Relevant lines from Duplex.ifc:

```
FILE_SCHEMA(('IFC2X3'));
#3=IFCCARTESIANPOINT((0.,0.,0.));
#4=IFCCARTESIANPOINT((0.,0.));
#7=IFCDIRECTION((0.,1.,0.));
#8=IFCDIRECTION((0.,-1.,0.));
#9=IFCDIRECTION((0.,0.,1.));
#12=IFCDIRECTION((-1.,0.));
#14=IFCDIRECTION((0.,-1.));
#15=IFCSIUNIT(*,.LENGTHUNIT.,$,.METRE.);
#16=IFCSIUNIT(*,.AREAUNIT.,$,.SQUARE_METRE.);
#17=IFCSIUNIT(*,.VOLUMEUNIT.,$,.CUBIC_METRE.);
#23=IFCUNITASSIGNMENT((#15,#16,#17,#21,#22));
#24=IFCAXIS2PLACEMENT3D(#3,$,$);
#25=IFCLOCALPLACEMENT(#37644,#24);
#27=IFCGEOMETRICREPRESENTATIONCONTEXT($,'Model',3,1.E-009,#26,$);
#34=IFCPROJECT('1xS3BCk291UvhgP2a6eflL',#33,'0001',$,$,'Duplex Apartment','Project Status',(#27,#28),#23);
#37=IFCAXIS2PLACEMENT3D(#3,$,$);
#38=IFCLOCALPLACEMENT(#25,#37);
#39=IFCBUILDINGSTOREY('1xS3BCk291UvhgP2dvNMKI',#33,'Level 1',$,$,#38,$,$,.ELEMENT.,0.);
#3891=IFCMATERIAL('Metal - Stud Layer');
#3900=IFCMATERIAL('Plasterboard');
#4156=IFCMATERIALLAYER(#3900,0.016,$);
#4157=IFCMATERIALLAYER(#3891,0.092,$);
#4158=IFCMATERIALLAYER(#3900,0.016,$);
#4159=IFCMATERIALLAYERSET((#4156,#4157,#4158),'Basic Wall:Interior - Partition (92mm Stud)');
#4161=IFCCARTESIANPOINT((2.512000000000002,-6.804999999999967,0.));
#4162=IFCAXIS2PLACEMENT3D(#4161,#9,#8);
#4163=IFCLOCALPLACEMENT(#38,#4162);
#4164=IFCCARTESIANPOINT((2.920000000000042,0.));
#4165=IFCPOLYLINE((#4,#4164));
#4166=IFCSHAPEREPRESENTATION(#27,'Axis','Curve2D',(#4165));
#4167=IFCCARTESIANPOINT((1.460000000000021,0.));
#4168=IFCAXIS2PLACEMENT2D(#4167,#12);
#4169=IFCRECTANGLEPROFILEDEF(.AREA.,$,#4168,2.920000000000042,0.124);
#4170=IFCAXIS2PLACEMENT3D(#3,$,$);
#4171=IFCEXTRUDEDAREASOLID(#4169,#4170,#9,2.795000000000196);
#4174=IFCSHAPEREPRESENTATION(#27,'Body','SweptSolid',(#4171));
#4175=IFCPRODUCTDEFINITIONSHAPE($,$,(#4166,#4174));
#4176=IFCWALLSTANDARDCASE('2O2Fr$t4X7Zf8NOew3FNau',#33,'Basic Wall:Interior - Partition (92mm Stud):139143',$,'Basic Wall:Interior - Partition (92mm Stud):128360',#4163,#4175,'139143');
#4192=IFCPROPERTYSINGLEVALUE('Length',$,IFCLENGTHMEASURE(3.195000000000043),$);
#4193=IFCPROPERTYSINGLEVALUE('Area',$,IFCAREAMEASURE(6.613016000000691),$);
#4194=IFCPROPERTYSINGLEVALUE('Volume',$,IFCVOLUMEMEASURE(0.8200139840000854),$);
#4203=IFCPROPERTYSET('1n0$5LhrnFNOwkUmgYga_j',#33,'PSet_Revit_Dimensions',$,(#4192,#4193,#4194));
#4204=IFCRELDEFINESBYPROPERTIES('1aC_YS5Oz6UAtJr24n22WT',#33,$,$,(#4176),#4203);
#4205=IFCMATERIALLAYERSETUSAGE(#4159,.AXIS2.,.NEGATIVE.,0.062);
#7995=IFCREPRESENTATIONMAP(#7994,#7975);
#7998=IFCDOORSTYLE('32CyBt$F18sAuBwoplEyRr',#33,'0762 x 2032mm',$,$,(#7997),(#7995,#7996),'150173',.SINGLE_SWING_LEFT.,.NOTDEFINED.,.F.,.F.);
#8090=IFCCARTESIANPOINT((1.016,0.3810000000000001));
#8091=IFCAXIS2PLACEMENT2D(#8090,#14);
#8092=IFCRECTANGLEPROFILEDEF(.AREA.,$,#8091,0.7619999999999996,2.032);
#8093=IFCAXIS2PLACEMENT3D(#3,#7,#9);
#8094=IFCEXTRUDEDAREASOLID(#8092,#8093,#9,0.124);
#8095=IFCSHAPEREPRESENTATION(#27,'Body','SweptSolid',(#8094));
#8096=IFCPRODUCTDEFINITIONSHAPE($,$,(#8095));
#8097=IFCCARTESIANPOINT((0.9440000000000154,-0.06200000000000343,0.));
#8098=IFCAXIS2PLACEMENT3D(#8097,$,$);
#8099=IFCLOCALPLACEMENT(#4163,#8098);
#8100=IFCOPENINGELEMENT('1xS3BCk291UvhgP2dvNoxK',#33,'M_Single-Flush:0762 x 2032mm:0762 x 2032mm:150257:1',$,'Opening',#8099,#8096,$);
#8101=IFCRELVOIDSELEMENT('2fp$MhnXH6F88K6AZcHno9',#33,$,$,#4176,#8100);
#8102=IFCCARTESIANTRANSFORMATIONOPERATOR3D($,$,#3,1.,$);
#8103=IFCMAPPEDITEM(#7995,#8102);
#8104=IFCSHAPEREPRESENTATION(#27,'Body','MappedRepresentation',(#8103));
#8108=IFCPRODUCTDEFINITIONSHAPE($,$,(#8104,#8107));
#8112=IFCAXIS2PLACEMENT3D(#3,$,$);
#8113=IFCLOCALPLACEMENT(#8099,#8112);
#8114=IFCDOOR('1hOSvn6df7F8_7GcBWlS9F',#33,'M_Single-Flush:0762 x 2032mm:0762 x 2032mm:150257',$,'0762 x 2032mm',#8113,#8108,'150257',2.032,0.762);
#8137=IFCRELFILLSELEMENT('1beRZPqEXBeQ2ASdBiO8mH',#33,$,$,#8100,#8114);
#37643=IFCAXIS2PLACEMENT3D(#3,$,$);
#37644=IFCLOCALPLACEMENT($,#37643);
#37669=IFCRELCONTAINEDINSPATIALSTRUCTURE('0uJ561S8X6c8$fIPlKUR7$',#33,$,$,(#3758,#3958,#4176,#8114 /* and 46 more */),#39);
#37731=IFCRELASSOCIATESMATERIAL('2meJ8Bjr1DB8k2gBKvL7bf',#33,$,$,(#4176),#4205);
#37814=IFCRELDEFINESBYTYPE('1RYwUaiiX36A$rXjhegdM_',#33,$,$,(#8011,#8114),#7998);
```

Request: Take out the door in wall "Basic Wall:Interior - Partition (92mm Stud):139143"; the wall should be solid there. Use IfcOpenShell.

```python
import ifcopenshell
import ifcopenshell.api.feature
import ifcopenshell.api.pset
import ifcopenshell.api.root
import ifcopenshell.geom
import ifcopenshell.util.element
import ifcopenshell.util.shape
import ifcopenshell.util.unit

model = ifcopenshell.open("Duplex.ifc")
area_scale = ifcopenshell.util.unit.calculate_unit_scale(model, "AREAUNIT")
volume_scale = ifcopenshell.util.unit.calculate_unit_scale(model, "VOLUMEUNIT")
settings = ifcopenshell.geom.settings()


def volume(element):
    """Net volume in cubic metres, openings subtracted."""
    shape = ifcopenshell.geom.create_shape(settings, element)
    return ifcopenshell.util.shape.get_volume(shape.geometry)


door = model.by_guid("1hOSvn6df7F8_7GcBWlS9F")
opening = door.FillsVoids[0].RelatingOpeningElement
wall = opening.VoidsElements[0].RelatingBuildingElement
before = volume(wall)

ifcopenshell.api.root.remove_product(model, product=door)
ifcopenshell.api.feature.remove_feature(model, feature=opening)

after = volume(wall)
thickness = 0.124  # wall thickness in metres

# Update the wall's stored quantities.
pset = model.by_id(ifcopenshell.util.element.get_pset(wall, "PSet_Revit_Dimensions", should_inherit=False)["id"])
ifcopenshell.api.pset.edit_pset(model, pset=pset, properties={
    "Area": model.create_entity("IfcAreaMeasure", after / thickness / area_scale),
    "Volume": model.create_entity("IfcVolumeMeasure", after / volume_scale),
})

print(f"wall volume {before:.3f} -> {after:.3f} m3")

model.write("Duplex_v2.ifc")
```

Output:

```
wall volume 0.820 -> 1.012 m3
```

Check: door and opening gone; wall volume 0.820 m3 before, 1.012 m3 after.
